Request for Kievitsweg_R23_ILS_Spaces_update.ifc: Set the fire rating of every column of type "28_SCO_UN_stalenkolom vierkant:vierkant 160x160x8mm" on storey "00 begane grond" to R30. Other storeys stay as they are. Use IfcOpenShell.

First a look at what the model holds.

```python
import ifcopenshell
import ifcopenshell.util.element

model = ifcopenshell.open("Kievitsweg_R23_ILS_Spaces_update.ifc")
print(model.schema)
storey = next(s for s in model.by_type("IfcBuildingStorey") if s.Name == "00 begane grond")
columns = [e for e in ifcopenshell.util.element.get_decomposition(storey) if e.is_a("IfcColumn")]
seen = {}
for e in columns:
    element_type = ifcopenshell.util.element.get_type(e)
    key = (element_type.Name if element_type != e and element_type else None, ifcopenshell.util.element.get_pset(e, "Pset_ColumnCommon", "FireRating"))
    seen[key] = seen.get(key, 0) + 1
for (name, value), count in sorted(seen.items(), key=str):
    print(count, "x", name, "|", value)
```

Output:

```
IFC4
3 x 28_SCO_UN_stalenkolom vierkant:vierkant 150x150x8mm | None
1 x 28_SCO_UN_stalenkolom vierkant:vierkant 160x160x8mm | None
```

```python
import ifcopenshell
import ifcopenshell.api.pset
import ifcopenshell.util.element

model = ifcopenshell.open("Kievitsweg_R23_ILS_Spaces_update.ifc")

storey = next(s for s in model.by_type("IfcBuildingStorey") if s.Name == "00 begane grond")
columns = [e for e in ifcopenshell.util.element.get_decomposition(storey) if e.is_a("IfcColumn")]

count = 0
for e in columns:
    element_type = ifcopenshell.util.element.get_type(e)
    if element_type in (None, e) or element_type.Name != "28_SCO_UN_stalenkolom vierkant:vierkant 160x160x8mm":
        continue
    # add_pset returns the element's existing set when there is one.
    pset = ifcopenshell.api.pset.add_pset(model, product=e, name="Pset_ColumnCommon")
    ifcopenshell.api.pset.edit_pset(model, pset=pset, properties={"FireRating": "R30"})
    count += 1

print(count, "columns updated")

model.write("Kievitsweg_R23_ILS_Spaces_update_v2.ifc")
```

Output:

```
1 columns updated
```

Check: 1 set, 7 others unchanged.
